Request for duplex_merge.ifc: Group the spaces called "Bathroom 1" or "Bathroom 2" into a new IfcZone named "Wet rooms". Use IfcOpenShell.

First a look at what the model holds.

```python
import ifcopenshell

model = ifcopenshell.open("duplex_merge.ifc")
print(model.schema)
seen = {}
for space in model.by_type("IfcSpace"):
    seen[space.LongName] = seen.get(space.LongName, 0) + 1
for name, count in sorted(seen.items(), key=str):
    print(count, "x", name)
print("zones:", [z.Name for z in model.by_type("IfcZone")][:20])
```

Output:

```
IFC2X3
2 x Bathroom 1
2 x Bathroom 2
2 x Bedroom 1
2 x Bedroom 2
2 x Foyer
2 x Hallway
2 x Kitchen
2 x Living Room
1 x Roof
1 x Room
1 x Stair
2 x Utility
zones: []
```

```python
import ifcopenshell
import ifcopenshell.api.group
import ifcopenshell.api.root

model = ifcopenshell.open("duplex_merge.ifc")

names = {"Bathroom 1", "Bathroom 2"}
spaces = [s for s in model.by_type("IfcSpace") if s.LongName in names]

zone = ifcopenshell.api.root.create_entity(model, ifc_class="IfcZone", name="Wet rooms")
ifcopenshell.api.group.assign_group(model, products=spaces, group=zone)
print(len(spaces), "spaces in", zone.Name)

model.write("duplex_merge_rev.ifc")
```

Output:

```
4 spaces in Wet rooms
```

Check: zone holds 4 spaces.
